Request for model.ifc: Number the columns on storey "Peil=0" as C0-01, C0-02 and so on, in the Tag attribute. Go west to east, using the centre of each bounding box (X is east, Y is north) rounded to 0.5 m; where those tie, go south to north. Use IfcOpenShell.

First a look at what the model holds.

```python
import ifcopenshell
import ifcopenshell.util.element
import ifcopenshell.util.placement

model = ifcopenshell.open("model.ifc")
print(model.schema)
storey = next(s for s in model.by_type("IfcBuildingStorey") if s.Name == "Peil=0")
columns = [e for e in ifcopenshell.util.element.get_decomposition(storey) if e.is_a("IfcColumn")]
for e in sorted(columns, key=lambda e: e.id()):
    origin = ifcopenshell.util.placement.get_local_placement(e.ObjectPlacement)[:3, 3]
    print(e.id(), e.Tag, e.Name, origin.round(2) + 0.0, sep=" | ")
```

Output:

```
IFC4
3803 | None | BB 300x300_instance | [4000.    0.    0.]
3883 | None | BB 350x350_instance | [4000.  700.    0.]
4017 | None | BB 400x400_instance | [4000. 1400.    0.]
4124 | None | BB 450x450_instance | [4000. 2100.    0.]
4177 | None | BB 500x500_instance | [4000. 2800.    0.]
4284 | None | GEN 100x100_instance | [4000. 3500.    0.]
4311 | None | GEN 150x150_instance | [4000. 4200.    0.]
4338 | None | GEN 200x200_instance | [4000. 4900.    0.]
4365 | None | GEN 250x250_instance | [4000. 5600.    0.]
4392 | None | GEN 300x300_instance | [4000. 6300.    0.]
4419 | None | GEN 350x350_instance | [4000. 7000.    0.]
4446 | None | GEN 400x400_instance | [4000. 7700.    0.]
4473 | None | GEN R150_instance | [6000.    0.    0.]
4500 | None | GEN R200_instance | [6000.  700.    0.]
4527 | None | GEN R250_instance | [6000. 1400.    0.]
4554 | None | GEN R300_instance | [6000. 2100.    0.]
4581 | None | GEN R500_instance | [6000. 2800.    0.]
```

```python
import ifcopenshell
import ifcopenshell.geom
import ifcopenshell.util.element
import ifcopenshell.util.shape

model = ifcopenshell.open("model.ifc")
settings = ifcopenshell.geom.settings()
settings.set("use-world-coords", True)


def centre(element):
    shape = ifcopenshell.geom.create_shape(settings, element)
    return ifcopenshell.util.shape.get_bbox_centroid(shape.geometry)


storey = next(s for s in model.by_type("IfcBuildingStorey") if s.Name == "Peil=0")
columns = [e for e in ifcopenshell.util.element.get_decomposition(storey) if e.is_a("IfcColumn")]

# Insertion points can sit at a corner or the storey origin, so sort by the geometry (in metres).
centres = {e: centre(e) for e in columns}
columns.sort(key=lambda e: (round(centres[e][0] / 0.5), centres[e][1]))

for i, e in enumerate(columns, start=1):
    number = f"C0-{i:02d}"
    e.Tag = number
    print(e.id(), number)

model.write("model_updated.ifc")
```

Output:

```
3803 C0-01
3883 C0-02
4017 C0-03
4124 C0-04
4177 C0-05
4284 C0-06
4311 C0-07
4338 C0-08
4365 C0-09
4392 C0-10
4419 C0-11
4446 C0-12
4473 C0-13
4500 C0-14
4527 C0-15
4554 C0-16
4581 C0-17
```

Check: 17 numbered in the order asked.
